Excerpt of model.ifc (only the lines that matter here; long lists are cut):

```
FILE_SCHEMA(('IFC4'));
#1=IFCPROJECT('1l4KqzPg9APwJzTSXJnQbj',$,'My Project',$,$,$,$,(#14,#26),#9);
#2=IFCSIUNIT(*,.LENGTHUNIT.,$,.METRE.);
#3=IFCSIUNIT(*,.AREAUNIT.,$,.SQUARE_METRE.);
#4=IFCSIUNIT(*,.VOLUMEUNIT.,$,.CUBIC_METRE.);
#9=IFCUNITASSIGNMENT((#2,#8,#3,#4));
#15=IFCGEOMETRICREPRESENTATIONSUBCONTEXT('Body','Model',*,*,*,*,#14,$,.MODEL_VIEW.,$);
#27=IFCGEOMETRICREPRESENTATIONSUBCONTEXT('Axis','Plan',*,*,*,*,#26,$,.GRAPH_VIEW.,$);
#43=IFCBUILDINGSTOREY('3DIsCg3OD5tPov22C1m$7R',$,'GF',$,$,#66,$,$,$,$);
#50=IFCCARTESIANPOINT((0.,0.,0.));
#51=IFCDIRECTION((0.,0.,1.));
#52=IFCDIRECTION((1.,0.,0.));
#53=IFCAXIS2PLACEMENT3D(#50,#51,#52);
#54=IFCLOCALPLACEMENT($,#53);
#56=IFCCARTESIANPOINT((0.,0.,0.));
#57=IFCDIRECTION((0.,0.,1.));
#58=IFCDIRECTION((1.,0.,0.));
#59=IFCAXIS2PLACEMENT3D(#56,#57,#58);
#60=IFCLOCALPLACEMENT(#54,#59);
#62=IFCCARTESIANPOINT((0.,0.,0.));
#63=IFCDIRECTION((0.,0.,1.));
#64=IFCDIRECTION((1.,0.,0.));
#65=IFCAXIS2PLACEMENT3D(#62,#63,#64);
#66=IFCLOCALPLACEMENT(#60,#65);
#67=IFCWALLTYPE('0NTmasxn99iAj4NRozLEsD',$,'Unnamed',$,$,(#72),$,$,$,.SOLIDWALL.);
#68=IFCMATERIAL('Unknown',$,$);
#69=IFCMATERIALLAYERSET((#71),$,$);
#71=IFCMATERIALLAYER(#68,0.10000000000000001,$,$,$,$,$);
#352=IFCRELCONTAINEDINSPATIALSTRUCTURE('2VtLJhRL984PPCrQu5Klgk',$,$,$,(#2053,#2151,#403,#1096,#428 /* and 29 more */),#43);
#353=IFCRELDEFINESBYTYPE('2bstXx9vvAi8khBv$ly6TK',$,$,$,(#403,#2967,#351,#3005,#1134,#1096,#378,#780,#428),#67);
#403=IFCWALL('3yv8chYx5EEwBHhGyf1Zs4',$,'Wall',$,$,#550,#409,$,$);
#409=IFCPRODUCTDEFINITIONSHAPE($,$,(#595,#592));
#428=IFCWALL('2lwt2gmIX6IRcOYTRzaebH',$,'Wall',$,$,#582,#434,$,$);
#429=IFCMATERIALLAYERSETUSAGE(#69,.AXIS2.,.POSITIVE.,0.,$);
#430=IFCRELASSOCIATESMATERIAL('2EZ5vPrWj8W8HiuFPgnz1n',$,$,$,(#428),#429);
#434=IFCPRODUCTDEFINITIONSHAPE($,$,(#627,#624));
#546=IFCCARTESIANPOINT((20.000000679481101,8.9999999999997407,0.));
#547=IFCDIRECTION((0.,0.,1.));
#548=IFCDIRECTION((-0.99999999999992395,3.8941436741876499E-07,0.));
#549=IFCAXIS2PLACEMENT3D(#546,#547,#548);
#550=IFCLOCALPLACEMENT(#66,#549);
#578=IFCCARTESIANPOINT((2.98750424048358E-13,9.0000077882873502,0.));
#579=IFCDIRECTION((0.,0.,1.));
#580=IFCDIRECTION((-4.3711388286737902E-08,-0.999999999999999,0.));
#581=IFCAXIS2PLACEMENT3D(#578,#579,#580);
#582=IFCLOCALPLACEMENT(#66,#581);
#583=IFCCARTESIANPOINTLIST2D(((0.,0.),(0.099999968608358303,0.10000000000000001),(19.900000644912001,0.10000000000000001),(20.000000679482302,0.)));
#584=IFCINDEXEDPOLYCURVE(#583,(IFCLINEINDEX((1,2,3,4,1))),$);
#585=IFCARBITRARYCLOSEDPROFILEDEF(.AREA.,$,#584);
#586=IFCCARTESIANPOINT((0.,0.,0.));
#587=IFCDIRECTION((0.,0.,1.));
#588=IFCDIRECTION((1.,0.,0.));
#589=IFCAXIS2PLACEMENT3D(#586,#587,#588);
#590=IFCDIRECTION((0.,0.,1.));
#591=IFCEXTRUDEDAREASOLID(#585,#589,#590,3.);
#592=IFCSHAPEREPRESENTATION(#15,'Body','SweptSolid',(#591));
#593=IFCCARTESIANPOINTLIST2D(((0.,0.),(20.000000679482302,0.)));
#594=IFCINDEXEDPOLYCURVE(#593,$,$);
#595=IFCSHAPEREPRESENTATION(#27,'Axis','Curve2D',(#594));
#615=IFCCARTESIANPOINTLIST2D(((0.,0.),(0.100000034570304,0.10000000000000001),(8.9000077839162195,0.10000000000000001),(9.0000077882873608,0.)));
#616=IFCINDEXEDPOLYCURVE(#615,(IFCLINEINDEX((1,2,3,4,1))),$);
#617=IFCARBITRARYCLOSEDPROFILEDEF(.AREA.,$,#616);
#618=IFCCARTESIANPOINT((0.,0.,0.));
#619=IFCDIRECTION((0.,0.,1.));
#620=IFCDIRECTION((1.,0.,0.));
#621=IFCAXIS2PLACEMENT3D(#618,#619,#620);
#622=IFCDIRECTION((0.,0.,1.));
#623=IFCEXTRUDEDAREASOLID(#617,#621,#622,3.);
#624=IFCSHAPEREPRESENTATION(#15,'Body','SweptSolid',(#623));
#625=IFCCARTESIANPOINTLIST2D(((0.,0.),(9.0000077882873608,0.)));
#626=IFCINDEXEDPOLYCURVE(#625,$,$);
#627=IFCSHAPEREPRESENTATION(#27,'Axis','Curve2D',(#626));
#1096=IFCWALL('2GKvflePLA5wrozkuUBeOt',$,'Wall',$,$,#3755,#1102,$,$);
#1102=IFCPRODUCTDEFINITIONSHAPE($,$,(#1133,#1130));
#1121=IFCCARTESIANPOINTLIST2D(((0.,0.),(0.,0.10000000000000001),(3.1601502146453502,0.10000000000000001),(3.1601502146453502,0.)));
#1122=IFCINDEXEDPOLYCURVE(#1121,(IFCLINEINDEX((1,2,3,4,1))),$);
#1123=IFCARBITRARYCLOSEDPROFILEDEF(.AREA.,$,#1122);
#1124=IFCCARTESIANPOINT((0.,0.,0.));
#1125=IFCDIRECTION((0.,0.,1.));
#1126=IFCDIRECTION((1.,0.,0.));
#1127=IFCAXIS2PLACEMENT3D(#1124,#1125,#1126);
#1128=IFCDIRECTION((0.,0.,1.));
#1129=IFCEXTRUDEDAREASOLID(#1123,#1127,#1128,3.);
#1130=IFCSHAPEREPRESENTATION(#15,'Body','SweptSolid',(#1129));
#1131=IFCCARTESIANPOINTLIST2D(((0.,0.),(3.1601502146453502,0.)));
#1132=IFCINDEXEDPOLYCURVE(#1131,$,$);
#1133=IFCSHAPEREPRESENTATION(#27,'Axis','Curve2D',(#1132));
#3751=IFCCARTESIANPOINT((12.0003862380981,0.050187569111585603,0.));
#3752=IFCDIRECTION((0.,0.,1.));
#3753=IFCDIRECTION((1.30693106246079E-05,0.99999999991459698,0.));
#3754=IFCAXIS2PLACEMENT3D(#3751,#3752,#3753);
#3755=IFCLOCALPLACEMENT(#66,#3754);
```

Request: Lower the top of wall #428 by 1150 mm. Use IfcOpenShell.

```python
import ifcopenshell
import ifcopenshell.geom
import ifcopenshell.util.representation
import ifcopenshell.util.shape

model = ifcopenshell.open("model.ifc")
settings = ifcopenshell.geom.settings()


def volume(element):
    """Net volume in cubic metres, openings subtracted."""
    shape = ifcopenshell.geom.create_shape(settings, element)
    return ifcopenshell.util.shape.get_volume(shape.geometry)


wall = model.by_guid("2lwt2gmIX6IRcOYTRzaebH")
before = volume(wall)

body = ifcopenshell.util.representation.get_representation(wall, "Model", "Body")
solid = body.Items[0]
old_height = solid.Depth
solid.Depth -= 1.15
after = volume(wall)

print(f"height {old_height:g} -> {solid.Depth:g}, volume {before:.3f} -> {after:.3f} m3")

model.write("model_updated.ifc")
```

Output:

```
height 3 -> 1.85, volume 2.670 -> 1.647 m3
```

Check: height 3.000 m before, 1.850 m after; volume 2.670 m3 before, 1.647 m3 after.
